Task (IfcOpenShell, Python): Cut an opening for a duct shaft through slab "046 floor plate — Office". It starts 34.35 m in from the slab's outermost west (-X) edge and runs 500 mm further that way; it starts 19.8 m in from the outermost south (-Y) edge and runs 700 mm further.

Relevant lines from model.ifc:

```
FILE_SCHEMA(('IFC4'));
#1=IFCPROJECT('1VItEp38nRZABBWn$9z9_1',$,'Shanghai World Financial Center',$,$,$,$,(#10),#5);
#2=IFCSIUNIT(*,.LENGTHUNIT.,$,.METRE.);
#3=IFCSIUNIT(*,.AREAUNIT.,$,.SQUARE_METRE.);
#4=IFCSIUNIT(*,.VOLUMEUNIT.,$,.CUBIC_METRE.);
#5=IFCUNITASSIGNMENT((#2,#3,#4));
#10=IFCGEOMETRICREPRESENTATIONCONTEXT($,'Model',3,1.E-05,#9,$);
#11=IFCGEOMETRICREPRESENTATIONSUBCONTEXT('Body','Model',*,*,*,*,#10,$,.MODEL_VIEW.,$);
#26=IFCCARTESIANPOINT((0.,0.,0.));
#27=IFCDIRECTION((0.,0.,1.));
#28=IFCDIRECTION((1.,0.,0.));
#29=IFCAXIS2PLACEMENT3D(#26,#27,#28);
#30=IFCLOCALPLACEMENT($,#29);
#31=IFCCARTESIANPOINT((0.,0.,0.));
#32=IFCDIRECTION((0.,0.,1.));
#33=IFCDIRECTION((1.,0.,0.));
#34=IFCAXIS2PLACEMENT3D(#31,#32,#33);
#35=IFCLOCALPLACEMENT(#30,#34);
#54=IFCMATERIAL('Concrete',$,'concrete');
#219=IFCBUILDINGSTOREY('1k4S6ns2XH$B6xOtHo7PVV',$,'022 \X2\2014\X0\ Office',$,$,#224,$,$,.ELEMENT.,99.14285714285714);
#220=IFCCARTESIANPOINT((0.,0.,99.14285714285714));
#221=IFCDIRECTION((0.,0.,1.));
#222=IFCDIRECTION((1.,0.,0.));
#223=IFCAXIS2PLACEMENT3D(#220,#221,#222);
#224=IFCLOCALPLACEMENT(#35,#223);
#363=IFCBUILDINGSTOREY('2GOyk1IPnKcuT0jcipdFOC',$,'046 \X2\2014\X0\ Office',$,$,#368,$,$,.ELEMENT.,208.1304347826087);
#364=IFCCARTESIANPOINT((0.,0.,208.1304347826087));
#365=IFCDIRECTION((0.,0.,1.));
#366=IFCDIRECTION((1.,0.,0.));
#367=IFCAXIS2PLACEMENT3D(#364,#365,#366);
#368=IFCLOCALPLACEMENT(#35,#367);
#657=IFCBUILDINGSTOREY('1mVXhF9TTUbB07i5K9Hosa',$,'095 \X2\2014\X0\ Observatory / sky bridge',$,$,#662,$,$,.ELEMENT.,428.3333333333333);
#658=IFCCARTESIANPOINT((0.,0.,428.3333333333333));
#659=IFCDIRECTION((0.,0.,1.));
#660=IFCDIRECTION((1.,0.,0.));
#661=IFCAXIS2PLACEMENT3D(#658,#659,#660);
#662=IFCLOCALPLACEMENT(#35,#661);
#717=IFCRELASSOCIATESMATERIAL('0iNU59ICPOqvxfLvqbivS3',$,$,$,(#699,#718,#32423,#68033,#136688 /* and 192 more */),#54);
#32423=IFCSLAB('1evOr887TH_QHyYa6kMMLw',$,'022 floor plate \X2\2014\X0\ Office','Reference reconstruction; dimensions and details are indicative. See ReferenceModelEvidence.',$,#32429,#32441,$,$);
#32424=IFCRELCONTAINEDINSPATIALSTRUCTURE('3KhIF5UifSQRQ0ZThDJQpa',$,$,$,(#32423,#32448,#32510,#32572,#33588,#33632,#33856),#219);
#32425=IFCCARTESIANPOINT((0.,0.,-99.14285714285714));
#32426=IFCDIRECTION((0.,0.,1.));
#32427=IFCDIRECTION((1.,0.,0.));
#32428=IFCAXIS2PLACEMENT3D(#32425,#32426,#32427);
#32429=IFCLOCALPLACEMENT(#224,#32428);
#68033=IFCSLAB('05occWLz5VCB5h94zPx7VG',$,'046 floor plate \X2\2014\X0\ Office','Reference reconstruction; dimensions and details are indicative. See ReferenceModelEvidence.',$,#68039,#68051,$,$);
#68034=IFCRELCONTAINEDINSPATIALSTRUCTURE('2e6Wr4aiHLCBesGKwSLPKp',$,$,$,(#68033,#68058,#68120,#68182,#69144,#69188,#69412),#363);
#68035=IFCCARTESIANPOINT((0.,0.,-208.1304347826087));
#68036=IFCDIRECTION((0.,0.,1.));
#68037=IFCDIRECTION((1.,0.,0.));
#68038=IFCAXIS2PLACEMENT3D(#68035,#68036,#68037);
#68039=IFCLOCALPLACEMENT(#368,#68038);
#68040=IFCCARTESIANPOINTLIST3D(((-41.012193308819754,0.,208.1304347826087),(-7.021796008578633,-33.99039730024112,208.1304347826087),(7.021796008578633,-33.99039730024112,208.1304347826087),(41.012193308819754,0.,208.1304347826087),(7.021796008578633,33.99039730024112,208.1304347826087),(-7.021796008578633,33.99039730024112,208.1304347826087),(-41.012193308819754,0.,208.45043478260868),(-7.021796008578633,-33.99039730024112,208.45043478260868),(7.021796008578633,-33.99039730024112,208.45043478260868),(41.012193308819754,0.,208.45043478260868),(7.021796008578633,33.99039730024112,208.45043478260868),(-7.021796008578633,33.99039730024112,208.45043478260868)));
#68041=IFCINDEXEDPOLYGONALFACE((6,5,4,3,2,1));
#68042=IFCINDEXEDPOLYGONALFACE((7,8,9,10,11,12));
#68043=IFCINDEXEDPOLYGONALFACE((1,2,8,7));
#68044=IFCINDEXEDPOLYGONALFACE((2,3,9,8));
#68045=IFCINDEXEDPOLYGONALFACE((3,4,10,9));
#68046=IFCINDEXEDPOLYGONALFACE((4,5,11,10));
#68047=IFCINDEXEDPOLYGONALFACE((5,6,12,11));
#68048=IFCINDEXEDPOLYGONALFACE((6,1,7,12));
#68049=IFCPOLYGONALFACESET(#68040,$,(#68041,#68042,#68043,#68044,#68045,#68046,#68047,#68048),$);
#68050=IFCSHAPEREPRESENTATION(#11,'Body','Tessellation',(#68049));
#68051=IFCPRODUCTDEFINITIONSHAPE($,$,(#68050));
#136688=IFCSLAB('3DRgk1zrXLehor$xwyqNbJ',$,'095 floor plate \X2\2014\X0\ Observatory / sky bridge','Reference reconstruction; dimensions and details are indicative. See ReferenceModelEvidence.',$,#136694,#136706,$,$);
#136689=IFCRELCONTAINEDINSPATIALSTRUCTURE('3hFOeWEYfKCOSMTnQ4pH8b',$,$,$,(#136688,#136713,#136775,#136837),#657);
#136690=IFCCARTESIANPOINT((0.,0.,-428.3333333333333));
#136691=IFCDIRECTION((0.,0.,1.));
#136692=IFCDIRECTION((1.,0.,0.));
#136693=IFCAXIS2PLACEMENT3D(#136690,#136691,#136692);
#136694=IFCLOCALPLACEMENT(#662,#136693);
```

```python
import numpy as np
import ifcopenshell
import ifcopenshell.api.feature
import ifcopenshell.api.geometry
import ifcopenshell.api.root
import ifcopenshell.geom
import ifcopenshell.util.placement
import ifcopenshell.util.representation
import ifcopenshell.util.shape
import ifcopenshell.util.unit

model = ifcopenshell.open("model.ifc")
unit_scale = ifcopenshell.util.unit.calculate_unit_scale(model)
settings = ifcopenshell.geom.settings()


def volume(element):
    """Net volume in cubic metres, openings subtracted."""
    shape = ifcopenshell.geom.create_shape(settings, element)
    return ifcopenshell.util.shape.get_volume(shape.geometry)


slab = model.by_guid("05occWLz5VCB5h94zPx7VG")
before = volume(slab)

# Extent in the slab's own axes, in metres. The edges named are its -X and -Y sides.
slab_shape = ifcopenshell.geom.create_shape(settings, slab)
vertices = ifcopenshell.util.shape.get_vertices(slab_shape.geometry)
x_min, y_min, bottom = vertices.min(axis=0)
top = vertices[:, 2].max()

opening = ifcopenshell.api.root.create_entity(model, ifc_class="IfcOpeningElement", name="Duct shaft opening", predefined_type="OPENING")
context = ifcopenshell.util.representation.get_context(model, "Model", "Body", "MODEL_VIEW")
width, depth = 0.5, 0.7
outline = [(0.0, 0.0), (width, 0.0), (width, depth), (0.0, depth), (0.0, 0.0)]
# Overshoot both faces by 50 mm so the cut is clean.
shape = ifcopenshell.api.geometry.add_slab_representation(
    model, context=context, depth=top - bottom + 0.1, polyline=outline
)
ifcopenshell.api.geometry.assign_representation(model, product=opening, representation=shape)

matrix = ifcopenshell.util.placement.get_local_placement(slab.ObjectPlacement)
matrix[:, 3] = matrix @ np.append(np.array([x_min + 34.35, y_min + 19.8, bottom - 0.05]) / unit_scale, 1.0)
ifcopenshell.api.geometry.edit_object_placement(model, product=opening, matrix=matrix, is_si=False)
ifcopenshell.api.feature.add_feature(model, feature=opening, element=slab)

after = volume(slab)

print(f"slab volume {before:.3f} -> {after:.3f} m3")

model.write("model_rev.ifc")
```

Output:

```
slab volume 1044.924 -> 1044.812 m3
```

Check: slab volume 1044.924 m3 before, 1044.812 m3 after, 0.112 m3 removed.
